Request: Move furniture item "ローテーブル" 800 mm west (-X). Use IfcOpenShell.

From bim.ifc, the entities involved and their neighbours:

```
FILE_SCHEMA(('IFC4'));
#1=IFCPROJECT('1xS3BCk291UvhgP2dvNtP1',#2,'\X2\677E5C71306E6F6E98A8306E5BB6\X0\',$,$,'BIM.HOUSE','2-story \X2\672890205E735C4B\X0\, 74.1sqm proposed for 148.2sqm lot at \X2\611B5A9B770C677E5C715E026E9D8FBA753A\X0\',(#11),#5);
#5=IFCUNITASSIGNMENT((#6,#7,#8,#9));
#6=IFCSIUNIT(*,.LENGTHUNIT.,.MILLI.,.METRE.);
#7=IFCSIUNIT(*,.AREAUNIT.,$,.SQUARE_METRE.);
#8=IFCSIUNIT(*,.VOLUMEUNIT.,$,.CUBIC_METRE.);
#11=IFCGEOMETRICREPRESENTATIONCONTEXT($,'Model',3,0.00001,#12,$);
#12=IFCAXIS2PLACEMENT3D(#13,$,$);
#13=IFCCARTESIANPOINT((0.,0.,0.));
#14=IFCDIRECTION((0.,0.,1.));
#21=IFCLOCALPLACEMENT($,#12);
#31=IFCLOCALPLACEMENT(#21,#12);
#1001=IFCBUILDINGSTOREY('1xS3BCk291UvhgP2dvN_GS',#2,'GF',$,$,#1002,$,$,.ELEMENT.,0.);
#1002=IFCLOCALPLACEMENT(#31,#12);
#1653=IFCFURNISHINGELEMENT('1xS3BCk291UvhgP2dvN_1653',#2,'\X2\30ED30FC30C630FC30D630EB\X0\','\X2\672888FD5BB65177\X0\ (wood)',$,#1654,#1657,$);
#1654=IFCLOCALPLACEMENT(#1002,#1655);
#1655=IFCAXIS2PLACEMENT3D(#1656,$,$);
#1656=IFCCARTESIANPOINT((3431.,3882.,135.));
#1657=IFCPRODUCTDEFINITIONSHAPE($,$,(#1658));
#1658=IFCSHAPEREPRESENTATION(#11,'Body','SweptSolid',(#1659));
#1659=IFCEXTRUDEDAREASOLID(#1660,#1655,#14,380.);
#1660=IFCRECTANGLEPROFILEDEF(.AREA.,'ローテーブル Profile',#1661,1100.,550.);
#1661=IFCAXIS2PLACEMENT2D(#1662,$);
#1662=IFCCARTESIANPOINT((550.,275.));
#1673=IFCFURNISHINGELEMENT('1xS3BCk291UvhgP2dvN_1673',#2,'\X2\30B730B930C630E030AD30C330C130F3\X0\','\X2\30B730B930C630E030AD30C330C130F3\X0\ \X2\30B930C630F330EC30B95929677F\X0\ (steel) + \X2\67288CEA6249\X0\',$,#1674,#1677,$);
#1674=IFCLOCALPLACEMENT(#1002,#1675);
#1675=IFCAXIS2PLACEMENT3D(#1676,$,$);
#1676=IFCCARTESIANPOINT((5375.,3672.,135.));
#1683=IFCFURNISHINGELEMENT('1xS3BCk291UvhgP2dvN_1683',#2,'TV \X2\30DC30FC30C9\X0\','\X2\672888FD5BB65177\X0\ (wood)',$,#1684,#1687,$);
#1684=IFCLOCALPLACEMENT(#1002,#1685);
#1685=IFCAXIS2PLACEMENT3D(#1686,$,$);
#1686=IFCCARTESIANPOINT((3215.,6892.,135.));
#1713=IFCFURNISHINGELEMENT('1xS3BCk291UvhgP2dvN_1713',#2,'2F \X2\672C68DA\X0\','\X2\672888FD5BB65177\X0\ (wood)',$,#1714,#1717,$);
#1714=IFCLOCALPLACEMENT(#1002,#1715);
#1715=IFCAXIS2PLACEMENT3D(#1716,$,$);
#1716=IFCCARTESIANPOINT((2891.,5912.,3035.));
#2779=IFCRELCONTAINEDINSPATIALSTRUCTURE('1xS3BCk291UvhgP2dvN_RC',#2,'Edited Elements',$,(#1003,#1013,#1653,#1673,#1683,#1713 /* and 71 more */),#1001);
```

```python
import ifcopenshell
import ifcopenshell.api.geometry
import ifcopenshell.util.placement

model = ifcopenshell.open("bim.ifc")

item = model.by_guid("1xS3BCk291UvhgP2dvN_1653")
matrix = ifcopenshell.util.placement.get_local_placement(item.ObjectPlacement)
matrix[0, 3] -= 800.0
ifcopenshell.api.geometry.edit_object_placement(model, product=item, matrix=matrix, is_si=False)

print(ifcopenshell.util.placement.get_local_placement(item.ObjectPlacement).round(3) + 0.0)

model.write("bim_edited.ifc")
```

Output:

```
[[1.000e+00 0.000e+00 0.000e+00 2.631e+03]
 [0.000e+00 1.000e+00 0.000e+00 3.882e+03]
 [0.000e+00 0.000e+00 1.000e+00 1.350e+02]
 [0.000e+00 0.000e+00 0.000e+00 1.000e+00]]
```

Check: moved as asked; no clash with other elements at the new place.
